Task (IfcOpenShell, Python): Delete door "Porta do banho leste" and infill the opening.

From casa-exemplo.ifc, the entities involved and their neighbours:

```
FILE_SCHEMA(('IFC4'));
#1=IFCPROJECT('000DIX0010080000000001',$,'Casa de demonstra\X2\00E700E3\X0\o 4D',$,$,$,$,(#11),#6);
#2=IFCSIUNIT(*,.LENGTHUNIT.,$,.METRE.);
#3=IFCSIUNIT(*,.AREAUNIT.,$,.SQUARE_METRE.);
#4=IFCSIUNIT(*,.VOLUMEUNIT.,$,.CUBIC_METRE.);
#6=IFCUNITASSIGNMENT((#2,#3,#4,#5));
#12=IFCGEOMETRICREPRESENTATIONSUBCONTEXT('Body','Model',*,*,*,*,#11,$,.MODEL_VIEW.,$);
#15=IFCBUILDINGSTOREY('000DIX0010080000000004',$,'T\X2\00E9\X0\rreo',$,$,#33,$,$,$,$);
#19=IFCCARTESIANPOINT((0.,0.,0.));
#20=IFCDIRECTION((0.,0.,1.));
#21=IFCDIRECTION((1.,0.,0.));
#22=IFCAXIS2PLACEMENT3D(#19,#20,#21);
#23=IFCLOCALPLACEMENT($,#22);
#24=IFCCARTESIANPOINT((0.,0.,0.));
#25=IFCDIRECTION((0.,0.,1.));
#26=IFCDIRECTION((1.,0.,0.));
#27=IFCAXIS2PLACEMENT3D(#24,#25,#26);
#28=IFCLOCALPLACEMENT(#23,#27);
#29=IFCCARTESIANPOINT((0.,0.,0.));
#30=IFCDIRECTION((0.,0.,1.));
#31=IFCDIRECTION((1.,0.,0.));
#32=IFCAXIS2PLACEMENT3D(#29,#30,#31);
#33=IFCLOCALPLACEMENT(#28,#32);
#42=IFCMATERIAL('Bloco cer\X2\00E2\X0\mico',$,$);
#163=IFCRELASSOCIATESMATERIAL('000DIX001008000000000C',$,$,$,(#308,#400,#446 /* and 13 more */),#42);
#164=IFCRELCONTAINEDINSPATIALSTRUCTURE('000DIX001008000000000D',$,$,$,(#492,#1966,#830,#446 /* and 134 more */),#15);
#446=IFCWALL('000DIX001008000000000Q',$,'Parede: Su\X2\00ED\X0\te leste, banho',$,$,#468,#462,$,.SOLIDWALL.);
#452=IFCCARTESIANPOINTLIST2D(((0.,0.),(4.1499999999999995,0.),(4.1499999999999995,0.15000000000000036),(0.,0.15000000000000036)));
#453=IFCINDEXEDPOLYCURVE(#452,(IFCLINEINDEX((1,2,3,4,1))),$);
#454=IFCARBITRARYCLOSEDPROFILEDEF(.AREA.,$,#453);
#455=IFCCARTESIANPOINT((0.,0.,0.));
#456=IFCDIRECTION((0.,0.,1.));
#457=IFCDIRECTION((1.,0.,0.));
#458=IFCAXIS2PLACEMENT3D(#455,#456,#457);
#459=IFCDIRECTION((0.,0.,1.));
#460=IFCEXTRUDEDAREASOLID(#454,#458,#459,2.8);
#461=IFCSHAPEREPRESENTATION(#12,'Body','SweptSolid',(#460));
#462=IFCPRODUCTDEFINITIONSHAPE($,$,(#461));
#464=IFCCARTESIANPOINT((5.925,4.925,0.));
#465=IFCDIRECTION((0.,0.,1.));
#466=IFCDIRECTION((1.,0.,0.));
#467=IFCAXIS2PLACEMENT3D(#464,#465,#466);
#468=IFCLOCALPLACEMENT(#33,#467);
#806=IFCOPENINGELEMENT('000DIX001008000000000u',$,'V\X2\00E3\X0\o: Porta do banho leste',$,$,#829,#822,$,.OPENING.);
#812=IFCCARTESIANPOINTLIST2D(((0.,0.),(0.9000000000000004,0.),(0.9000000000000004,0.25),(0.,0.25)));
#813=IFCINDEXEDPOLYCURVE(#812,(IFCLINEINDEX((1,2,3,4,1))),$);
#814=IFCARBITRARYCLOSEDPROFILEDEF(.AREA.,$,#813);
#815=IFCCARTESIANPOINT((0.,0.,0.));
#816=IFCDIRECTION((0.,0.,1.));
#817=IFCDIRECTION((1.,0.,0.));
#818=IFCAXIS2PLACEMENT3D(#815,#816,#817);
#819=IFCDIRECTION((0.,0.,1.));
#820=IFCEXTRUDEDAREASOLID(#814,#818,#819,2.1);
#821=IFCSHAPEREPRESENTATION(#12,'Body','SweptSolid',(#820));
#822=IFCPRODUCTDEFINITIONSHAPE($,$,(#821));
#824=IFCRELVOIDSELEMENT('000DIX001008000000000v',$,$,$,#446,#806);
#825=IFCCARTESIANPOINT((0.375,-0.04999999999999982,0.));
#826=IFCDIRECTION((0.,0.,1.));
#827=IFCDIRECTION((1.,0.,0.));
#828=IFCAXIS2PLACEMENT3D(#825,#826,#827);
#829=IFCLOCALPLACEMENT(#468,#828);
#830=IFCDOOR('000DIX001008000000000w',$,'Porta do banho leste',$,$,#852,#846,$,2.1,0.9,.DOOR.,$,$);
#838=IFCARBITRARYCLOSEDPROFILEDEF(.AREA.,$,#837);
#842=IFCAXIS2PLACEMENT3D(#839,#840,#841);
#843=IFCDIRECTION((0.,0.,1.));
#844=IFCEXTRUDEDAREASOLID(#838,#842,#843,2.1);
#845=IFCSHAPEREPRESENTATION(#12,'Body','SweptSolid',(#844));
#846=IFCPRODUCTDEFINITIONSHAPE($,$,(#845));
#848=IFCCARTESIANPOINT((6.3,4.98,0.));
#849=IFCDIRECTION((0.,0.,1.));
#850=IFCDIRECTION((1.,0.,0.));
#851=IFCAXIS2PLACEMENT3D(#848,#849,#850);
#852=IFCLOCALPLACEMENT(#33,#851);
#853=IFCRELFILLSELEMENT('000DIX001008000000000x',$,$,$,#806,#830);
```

```python
import ifcopenshell
import ifcopenshell.api.feature
import ifcopenshell.api.root
import ifcopenshell.geom
import ifcopenshell.util.shape

model = ifcopenshell.open("casa-exemplo.ifc")
settings = ifcopenshell.geom.settings()


def volume(element):
    """Net volume in cubic metres, openings subtracted."""
    shape = ifcopenshell.geom.create_shape(settings, element)
    return ifcopenshell.util.shape.get_volume(shape.geometry)


door = model.by_guid("000DIX001008000000000w")
opening = door.FillsVoids[0].RelatingOpeningElement
wall = opening.VoidsElements[0].RelatingBuildingElement
before = volume(wall)

ifcopenshell.api.root.remove_product(model, product=door)
ifcopenshell.api.feature.remove_feature(model, feature=opening)

after = volume(wall)

print(f"wall volume {before:.3f} -> {after:.3f} m3")

model.write("casa-exemplo_rev.ifc")
```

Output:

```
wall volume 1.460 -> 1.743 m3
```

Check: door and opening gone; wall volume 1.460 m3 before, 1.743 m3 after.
